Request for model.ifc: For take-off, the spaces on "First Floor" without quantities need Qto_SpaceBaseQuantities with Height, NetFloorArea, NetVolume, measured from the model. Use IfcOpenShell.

First a look at what the model holds.

```python
import ifcopenshell
import ifcopenshell.util.element
import ifcopenshell.util.unit

model = ifcopenshell.open("model.ifc")
print(model.schema)
for unit_type in ("LENGTHUNIT", "AREAUNIT", "VOLUMEUNIT"):
    print(unit_type, ifcopenshell.util.unit.calculate_unit_scale(model, unit_type))
storey = next(s for s in model.by_type("IfcBuildingStorey") if s.Name == "First Floor")
spaces = [e for e in ifcopenshell.util.element.get_decomposition(storey) if e.is_a("IfcSpace")]
for e in sorted(spaces, key=lambda e: e.id()):
    print(e.id(), e.is_a(), e.Name, list(ifcopenshell.util.element.get_psets(e, qtos_only=True)), sep=" | ")
```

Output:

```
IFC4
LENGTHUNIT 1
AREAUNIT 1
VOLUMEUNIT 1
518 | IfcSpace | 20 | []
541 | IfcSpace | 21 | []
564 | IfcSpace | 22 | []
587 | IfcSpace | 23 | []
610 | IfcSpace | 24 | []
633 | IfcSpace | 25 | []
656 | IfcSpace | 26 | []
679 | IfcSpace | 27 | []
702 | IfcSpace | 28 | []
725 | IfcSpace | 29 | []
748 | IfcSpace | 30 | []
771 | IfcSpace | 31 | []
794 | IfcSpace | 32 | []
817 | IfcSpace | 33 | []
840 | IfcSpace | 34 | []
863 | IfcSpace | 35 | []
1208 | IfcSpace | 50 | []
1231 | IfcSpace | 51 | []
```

```python
import ifcopenshell
import ifcopenshell.api.pset
import ifcopenshell.geom
import ifcopenshell.util.element
import ifcopenshell.util.shape
import ifcopenshell.util.unit

model = ifcopenshell.open("model.ifc")
unit_scale = ifcopenshell.util.unit.calculate_unit_scale(model)
area_scale = ifcopenshell.util.unit.calculate_unit_scale(model, "AREAUNIT")
volume_scale = ifcopenshell.util.unit.calculate_unit_scale(model, "VOLUMEUNIT")
settings = ifcopenshell.geom.settings()

storey = next(s for s in model.by_type("IfcBuildingStorey") if s.Name == "First Floor")
spaces = [e for e in ifcopenshell.util.element.get_decomposition(storey) if e.is_a("IfcSpace")]

for e in sorted(spaces, key=lambda e: e.id()):
    if ifcopenshell.util.element.get_psets(e, qtos_only=True, should_inherit=False):
        continue
    # Geometry comes back in metres, in the element's own axes.
    shape = ifcopenshell.geom.create_shape(settings, e)
    values = {
        "Height": ifcopenshell.util.shape.get_z(shape.geometry) / unit_scale,
        "NetFloorArea": ifcopenshell.util.shape.get_footprint_area(shape.geometry) / area_scale,
        "NetVolume": ifcopenshell.util.shape.get_volume(shape.geometry) / volume_scale,
    }
    qto = ifcopenshell.api.pset.add_qto(model, product=e, name="Qto_SpaceBaseQuantities")
    ifcopenshell.api.pset.edit_qto(model, qto=qto, properties=values)
    print(e.id(), {k: round(v, 3) for k, v in values.items()})

model.write("model_v2.ifc")
```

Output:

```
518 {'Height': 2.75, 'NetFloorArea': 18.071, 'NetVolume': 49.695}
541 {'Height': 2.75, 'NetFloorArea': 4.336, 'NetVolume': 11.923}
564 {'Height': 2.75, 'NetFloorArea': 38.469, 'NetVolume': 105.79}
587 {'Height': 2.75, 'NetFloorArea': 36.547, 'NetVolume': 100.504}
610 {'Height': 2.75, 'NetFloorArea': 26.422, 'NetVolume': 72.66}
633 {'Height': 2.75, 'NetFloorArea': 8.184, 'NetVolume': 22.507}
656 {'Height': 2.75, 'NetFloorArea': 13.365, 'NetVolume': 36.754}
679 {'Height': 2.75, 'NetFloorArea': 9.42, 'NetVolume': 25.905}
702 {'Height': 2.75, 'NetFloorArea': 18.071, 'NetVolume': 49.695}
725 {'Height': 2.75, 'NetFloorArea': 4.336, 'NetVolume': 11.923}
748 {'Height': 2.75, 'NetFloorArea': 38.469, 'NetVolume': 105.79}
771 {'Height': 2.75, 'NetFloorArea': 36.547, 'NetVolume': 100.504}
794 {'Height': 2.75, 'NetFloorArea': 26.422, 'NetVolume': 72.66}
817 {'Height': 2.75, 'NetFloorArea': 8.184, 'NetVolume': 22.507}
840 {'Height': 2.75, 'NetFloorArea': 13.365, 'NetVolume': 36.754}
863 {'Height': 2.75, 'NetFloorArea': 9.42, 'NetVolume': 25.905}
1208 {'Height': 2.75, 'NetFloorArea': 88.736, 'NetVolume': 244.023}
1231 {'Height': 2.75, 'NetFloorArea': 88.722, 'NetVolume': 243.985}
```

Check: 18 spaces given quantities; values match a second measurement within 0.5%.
